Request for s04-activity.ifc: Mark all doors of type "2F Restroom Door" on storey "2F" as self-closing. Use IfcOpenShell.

First a look at what the model holds.

```python
import ifcopenshell
import ifcopenshell.util.element

model = ifcopenshell.open("s04-activity.ifc")
print(model.schema)
storey = next(s for s in model.by_type("IfcBuildingStorey") if s.Name == "2F")
doors = [e for e in ifcopenshell.util.element.get_decomposition(storey) if e.is_a("IfcDoor")]
seen = {}
for e in doors:
    element_type = ifcopenshell.util.element.get_type(e)
    key = (element_type.Name if element_type != e and element_type else None, ifcopenshell.util.element.get_pset(e, "Pset_DoorCommon", "SelfClosing"))
    seen[key] = seen.get(key, 0) + 1
for (name, value), count in sorted(seen.items(), key=str):
    print(count, "x", name, "|", value)
```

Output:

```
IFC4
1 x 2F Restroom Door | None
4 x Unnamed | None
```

```python
import ifcopenshell
import ifcopenshell.api.pset
import ifcopenshell.util.element

model = ifcopenshell.open("s04-activity.ifc")

storey = next(s for s in model.by_type("IfcBuildingStorey") if s.Name == "2F")
doors = [e for e in ifcopenshell.util.element.get_decomposition(storey) if e.is_a("IfcDoor")]

count = 0
for e in doors:
    element_type = ifcopenshell.util.element.get_type(e)
    if element_type in (None, e) or element_type.Name != "2F Restroom Door":
        continue
    # add_pset returns the element's existing set when there is one.
    pset = ifcopenshell.api.pset.add_pset(model, product=e, name="Pset_DoorCommon")
    ifcopenshell.api.pset.edit_pset(model, pset=pset, properties={"SelfClosing": True})
    count += 1

print(count, "doors updated")

model.write("s04-activity_edited.ifc")
```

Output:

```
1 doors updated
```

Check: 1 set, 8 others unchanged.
